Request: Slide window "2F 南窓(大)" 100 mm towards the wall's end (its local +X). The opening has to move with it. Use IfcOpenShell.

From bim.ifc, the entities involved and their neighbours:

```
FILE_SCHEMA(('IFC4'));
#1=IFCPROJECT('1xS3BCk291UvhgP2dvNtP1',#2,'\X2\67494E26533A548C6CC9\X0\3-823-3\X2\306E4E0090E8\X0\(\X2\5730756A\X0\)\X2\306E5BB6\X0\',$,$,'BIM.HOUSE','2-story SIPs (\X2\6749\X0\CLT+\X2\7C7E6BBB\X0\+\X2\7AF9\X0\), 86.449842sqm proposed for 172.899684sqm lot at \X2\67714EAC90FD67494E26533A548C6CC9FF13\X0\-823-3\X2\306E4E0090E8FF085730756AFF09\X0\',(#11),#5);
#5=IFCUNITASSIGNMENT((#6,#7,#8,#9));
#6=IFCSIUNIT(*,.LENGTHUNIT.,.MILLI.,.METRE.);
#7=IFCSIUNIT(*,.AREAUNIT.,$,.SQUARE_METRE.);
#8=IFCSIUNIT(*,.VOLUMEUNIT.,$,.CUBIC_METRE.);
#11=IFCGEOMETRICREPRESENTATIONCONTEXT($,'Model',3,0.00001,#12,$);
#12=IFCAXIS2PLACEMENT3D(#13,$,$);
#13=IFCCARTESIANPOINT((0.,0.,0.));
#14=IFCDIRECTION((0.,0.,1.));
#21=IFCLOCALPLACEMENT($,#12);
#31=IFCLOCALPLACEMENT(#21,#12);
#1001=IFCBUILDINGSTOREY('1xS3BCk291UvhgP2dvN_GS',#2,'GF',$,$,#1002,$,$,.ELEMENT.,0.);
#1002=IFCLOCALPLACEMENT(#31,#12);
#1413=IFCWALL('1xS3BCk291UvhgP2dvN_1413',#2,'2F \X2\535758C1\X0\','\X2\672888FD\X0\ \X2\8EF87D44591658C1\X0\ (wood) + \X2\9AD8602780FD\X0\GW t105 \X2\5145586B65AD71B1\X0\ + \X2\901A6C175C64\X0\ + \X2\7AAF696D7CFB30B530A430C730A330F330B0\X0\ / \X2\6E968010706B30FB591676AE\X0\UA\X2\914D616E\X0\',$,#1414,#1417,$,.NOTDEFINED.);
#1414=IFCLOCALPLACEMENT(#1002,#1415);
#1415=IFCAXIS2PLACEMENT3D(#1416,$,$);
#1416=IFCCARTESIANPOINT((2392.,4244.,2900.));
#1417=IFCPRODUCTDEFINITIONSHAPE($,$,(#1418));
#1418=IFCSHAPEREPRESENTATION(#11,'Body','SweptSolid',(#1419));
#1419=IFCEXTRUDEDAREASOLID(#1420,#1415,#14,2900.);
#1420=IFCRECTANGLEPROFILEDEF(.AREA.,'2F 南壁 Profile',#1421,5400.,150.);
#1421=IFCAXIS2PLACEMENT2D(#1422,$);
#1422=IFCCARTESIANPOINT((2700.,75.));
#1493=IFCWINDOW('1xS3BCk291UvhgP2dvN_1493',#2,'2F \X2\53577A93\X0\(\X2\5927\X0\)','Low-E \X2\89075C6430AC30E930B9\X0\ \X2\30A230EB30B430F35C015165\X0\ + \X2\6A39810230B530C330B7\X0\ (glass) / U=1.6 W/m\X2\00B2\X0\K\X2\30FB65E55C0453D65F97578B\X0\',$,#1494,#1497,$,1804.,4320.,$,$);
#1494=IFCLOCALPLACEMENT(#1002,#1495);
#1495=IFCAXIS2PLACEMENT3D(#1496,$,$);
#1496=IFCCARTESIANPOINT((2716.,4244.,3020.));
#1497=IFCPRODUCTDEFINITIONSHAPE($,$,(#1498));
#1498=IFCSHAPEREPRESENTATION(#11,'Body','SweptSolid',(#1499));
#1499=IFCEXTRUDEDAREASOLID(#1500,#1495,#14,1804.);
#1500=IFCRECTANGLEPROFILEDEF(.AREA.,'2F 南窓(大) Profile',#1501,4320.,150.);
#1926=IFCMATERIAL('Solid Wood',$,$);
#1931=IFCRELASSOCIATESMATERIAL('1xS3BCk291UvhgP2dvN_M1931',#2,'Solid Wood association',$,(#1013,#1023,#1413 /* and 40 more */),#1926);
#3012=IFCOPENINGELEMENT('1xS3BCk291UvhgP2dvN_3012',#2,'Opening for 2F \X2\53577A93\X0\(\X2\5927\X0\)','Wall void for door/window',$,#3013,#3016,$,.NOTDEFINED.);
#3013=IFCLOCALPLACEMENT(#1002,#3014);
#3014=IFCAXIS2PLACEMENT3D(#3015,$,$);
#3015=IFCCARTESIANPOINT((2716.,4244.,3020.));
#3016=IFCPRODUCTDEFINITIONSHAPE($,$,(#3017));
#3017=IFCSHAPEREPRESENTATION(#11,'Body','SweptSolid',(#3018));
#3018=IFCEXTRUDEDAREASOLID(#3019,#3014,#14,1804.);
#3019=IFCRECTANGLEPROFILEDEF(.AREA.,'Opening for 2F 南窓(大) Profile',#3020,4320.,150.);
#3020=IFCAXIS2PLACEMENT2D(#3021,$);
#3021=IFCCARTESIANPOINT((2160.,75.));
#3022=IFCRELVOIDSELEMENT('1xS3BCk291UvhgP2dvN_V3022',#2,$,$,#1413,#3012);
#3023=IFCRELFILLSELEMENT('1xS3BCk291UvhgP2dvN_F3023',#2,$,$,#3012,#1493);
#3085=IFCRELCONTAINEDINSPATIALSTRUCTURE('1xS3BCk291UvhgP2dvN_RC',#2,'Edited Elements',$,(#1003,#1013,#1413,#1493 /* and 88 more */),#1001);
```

```python
import ifcopenshell
import ifcopenshell.api.geometry
import ifcopenshell.util.placement

model = ifcopenshell.open("bim.ifc")

window = model.by_id(1493)
opening = window.FillsVoids[0].RelatingOpeningElement
wall = opening.VoidsElements[0].RelatingBuildingElement

wall_matrix = ifcopenshell.util.placement.get_local_placement(wall.ObjectPlacement)
shift = wall_matrix[:3, 0] * 100.0
before = ifcopenshell.util.placement.get_local_placement(window.ObjectPlacement)[:3, 3].copy()

# The window is not placed relative to its opening, so move both.
for product in (opening, window):
    matrix = ifcopenshell.util.placement.get_local_placement(product.ObjectPlacement)
    matrix[:3, 3] += shift
    ifcopenshell.api.geometry.edit_object_placement(model, product=product, matrix=matrix, is_si=False)

after = ifcopenshell.util.placement.get_local_placement(window.ObjectPlacement)[:3, 3]
print("window moved by", (after - before).round(3) + 0.0)

model.write("bim_edited.ifc")
```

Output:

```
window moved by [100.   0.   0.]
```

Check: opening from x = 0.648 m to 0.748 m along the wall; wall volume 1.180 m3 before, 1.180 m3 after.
